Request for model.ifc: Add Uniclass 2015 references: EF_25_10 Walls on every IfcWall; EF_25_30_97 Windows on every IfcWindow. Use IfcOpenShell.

First a look at what the model holds.

```python
import ifcopenshell

model = ifcopenshell.open("model.ifc")
print(model.schema)
print("classifications:", [c.Name for c in model.by_type("IfcClassification")])
for ifc_class in ("IfcDoor", "IfcRoof", "IfcStair", "IfcWall", "IfcWindow"):
    print(ifc_class, len(model.by_type(ifc_class)))
```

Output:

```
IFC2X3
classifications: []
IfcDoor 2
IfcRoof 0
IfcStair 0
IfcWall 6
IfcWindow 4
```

```python
import ifcopenshell
import ifcopenshell.api.classification

model = ifcopenshell.open("model.ifc")

# IFC2X3 requires Source and Edition and has no link from the project to the system.
system = model.create_entity("IfcClassification", Source="NBS", Edition="2015", Name="Uniclass 2015")

codes = {
    "IfcWall": ("EF_25_10", "Walls"),
    "IfcWindow": ("EF_25_30_97", "Windows"),
}
for ifc_class, (code, name) in codes.items():
    products = model.by_type(ifc_class)
    ifcopenshell.api.classification.add_reference(
        model, products=products, classification=system, identification=code, name=name
    )
    print(code, len(products))

model.write("model_rev.ifc")
```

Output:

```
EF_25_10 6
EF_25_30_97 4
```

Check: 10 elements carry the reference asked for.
